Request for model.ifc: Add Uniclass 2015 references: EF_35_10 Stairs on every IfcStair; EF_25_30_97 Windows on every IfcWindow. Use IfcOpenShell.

First a look at what the model holds.

```python
import ifcopenshell

model = ifcopenshell.open("model.ifc")
print(model.schema)
print("classifications:", [c.Name for c in model.by_type("IfcClassification")])
for ifc_class in ("IfcDoor", "IfcRoof", "IfcStair", "IfcWall", "IfcWindow"):
    print(ifc_class, len(model.by_type(ifc_class)))
```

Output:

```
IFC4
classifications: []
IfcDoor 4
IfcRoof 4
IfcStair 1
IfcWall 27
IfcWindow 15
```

```python
import ifcopenshell
import ifcopenshell.api.classification

model = ifcopenshell.open("model.ifc")

system = ifcopenshell.api.classification.add_classification(model, classification="Uniclass 2015")

codes = {
    "IfcStair": ("EF_35_10", "Stairs"),
    "IfcWindow": ("EF_25_30_97", "Windows"),
}
for ifc_class, (code, name) in codes.items():
    products = model.by_type(ifc_class)
    ifcopenshell.api.classification.add_reference(
        model, products=products, classification=system, identification=code, name=name
    )
    print(code, len(products))

model.write("model_updated.ifc")
```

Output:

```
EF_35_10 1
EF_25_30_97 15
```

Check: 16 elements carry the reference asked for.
